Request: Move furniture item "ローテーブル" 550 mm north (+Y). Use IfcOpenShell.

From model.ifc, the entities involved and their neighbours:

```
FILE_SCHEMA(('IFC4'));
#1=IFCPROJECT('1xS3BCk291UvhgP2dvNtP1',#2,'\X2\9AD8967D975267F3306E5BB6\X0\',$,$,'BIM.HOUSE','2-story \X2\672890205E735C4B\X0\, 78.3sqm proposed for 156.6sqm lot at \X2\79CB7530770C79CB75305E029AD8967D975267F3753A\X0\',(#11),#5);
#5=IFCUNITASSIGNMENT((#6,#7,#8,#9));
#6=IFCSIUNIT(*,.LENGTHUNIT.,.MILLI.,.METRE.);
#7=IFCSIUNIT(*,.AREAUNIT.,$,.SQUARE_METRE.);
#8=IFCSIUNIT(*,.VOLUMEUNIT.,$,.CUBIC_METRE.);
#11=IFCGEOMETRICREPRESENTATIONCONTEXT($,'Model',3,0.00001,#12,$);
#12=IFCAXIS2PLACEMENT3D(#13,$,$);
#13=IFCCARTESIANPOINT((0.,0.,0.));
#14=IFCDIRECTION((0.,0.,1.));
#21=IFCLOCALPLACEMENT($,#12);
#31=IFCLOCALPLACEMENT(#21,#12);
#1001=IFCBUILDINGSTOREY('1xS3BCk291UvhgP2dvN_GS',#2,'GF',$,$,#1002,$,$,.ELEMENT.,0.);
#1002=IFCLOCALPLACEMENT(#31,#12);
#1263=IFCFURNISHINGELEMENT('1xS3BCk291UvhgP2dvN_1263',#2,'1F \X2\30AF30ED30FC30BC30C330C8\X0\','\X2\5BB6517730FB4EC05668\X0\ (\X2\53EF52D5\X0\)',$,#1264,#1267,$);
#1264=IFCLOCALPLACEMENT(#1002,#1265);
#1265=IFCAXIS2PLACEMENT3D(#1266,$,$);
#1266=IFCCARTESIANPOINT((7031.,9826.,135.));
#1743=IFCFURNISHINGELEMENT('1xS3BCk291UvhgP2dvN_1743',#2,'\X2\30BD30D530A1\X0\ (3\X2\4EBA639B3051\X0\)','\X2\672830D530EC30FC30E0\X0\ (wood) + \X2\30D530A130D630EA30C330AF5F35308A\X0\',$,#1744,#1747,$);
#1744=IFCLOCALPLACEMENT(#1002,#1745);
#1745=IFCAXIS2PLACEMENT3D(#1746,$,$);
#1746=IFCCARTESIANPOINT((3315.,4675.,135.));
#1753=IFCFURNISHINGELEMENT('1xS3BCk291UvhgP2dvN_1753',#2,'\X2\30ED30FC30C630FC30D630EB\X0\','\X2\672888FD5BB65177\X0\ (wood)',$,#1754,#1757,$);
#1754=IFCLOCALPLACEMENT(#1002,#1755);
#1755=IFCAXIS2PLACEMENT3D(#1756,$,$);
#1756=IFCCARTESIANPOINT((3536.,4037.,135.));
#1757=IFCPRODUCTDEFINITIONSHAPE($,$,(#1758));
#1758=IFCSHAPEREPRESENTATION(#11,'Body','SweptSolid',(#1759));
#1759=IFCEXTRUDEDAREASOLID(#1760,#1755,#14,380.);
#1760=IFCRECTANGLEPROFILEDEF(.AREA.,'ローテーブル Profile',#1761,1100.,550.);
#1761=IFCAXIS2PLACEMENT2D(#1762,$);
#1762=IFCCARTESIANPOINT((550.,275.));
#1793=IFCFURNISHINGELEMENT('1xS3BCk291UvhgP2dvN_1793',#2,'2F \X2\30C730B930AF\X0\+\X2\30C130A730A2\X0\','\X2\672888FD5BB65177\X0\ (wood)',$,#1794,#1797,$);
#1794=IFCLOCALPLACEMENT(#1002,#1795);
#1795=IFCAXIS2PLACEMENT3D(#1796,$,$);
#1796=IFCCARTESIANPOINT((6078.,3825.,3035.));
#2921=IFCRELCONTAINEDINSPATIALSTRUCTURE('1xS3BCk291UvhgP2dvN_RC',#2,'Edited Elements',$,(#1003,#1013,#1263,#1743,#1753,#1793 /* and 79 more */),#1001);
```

```python
import ifcopenshell
import ifcopenshell.api.geometry
import ifcopenshell.util.placement
import ifcopenshell.util.unit

model = ifcopenshell.open("model.ifc")
unit_scale = ifcopenshell.util.unit.calculate_unit_scale(model)

item = model.by_guid("1xS3BCk291UvhgP2dvN_1753")
matrix = ifcopenshell.util.placement.get_local_placement(item.ObjectPlacement)
matrix[1, 3] += 0.55 / unit_scale
ifcopenshell.api.geometry.edit_object_placement(model, product=item, matrix=matrix, is_si=False)

print(ifcopenshell.util.placement.get_local_placement(item.ObjectPlacement).round(3) + 0.0)

model.write("model_v2.ifc")
```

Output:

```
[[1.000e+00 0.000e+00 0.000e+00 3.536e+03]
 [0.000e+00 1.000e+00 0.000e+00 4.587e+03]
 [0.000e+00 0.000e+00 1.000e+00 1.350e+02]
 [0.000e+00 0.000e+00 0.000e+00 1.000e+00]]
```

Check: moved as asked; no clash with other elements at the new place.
